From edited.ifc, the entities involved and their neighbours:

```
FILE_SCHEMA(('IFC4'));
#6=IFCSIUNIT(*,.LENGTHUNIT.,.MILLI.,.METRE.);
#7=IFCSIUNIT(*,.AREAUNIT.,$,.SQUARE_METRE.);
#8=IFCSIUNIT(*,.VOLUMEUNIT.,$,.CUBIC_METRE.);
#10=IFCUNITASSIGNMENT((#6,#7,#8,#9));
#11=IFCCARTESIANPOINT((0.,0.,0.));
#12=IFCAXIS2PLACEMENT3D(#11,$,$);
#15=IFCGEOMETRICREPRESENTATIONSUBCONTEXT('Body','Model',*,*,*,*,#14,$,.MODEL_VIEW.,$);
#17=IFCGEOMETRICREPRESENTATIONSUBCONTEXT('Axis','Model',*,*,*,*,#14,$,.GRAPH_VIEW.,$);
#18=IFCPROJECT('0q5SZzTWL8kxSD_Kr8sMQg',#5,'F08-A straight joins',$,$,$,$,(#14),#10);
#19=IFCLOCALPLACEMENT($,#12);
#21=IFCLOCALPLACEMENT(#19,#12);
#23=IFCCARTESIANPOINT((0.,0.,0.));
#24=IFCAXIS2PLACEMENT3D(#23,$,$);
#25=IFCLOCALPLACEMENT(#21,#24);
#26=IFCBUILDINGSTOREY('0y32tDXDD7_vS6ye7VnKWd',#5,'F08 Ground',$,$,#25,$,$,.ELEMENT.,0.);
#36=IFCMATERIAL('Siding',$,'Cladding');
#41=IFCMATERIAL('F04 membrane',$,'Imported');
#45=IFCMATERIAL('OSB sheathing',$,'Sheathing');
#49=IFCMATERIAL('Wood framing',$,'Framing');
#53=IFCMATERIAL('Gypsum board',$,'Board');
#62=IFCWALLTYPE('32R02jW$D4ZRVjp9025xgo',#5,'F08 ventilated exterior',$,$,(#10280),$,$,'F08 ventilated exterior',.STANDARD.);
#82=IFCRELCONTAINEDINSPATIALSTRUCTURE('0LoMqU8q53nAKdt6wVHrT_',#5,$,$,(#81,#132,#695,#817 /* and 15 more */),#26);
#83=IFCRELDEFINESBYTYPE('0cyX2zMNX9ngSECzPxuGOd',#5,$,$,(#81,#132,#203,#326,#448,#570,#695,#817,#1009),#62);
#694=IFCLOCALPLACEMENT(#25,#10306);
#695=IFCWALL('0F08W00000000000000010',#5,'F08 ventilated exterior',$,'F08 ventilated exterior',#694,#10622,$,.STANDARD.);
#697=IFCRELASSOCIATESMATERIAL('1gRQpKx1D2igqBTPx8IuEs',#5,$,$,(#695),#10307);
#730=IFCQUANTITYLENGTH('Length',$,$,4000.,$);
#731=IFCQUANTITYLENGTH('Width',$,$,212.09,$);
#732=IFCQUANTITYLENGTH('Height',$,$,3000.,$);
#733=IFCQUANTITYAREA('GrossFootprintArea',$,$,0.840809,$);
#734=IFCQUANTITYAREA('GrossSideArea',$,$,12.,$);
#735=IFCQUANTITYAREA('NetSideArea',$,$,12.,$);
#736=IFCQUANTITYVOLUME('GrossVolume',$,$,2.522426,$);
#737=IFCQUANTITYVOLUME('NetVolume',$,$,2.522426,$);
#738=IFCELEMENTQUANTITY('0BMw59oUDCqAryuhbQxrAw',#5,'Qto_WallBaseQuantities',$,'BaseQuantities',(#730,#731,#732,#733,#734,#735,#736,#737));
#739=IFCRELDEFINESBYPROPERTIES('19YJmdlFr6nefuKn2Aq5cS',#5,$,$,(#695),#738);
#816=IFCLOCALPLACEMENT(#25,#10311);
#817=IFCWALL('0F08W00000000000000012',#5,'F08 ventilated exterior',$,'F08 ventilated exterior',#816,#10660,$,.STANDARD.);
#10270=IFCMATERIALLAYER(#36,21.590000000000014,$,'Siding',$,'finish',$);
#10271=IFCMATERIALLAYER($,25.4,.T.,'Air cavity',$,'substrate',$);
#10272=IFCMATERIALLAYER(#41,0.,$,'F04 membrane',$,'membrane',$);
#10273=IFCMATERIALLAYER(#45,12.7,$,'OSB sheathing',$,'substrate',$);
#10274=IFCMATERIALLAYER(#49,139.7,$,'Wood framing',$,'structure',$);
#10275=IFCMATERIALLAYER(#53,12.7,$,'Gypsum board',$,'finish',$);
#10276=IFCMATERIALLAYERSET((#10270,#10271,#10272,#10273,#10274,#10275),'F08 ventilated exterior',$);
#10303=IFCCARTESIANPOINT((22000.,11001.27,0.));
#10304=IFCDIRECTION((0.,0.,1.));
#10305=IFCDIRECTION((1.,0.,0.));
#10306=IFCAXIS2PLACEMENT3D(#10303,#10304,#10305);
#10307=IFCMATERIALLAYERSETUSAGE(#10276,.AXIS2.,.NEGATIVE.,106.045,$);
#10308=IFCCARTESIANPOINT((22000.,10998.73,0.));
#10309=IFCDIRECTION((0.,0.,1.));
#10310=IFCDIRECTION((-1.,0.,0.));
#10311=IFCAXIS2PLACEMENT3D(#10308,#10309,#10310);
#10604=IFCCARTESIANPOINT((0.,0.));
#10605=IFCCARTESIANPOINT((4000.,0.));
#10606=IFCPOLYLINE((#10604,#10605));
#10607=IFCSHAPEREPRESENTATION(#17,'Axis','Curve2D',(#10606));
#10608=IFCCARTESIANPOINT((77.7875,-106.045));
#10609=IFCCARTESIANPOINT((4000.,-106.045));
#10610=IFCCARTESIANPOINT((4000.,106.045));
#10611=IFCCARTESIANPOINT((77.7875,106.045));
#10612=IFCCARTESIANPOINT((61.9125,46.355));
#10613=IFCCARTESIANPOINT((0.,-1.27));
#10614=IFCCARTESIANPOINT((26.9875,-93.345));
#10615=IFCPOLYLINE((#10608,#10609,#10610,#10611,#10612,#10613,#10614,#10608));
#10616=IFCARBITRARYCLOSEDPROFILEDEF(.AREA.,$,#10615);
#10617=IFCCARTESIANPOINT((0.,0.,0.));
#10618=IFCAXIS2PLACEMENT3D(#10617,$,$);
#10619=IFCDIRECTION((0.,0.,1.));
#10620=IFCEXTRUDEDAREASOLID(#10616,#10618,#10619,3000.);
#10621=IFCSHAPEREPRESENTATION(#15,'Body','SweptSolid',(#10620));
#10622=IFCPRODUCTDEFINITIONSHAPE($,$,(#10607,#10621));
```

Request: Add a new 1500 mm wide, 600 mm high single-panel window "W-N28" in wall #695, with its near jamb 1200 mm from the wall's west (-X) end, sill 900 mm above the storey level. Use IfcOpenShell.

```python
import numpy as np
import ifcopenshell
import ifcopenshell.api.feature
import ifcopenshell.api.geometry
import ifcopenshell.api.pset
import ifcopenshell.api.root
import ifcopenshell.api.spatial
import ifcopenshell.geom
import ifcopenshell.util.element
import ifcopenshell.util.placement
import ifcopenshell.util.representation
import ifcopenshell.util.shape
import ifcopenshell.util.unit

model = ifcopenshell.open("edited.ifc")
unit_scale = ifcopenshell.util.unit.calculate_unit_scale(model)
area_scale = ifcopenshell.util.unit.calculate_unit_scale(model, "AREAUNIT")
volume_scale = ifcopenshell.util.unit.calculate_unit_scale(model, "VOLUMEUNIT")
settings = ifcopenshell.geom.settings()


def volume(element):
    """Net volume in cubic metres, openings subtracted."""
    shape = ifcopenshell.geom.create_shape(settings, element)
    return ifcopenshell.util.shape.get_volume(shape.geometry)


wall = model.by_guid("0F08W00000000000000010")
storey = ifcopenshell.util.element.get_container(wall, ifc_class="IfcBuildingStorey")
context = ifcopenshell.util.representation.get_context(model, "Model", "Body", "MODEL_VIEW")
before = volume(wall)

width, height, from_end, sill = 1.5, 0.6, 1.2, 0.9  # metres

# The wall runs along its own X axis, and the end named is its -X end.
wall_shape = ifcopenshell.geom.create_shape(settings, wall)
x, y, z = ifcopenshell.util.shape.get_vertices(wall_shape.geometry).T
start = x.min() + from_end
face, thickness = float(y.min()), float(y.max() - y.min())
wall_matrix = ifcopenshell.util.placement.get_local_placement(wall.ObjectPlacement)
level = ifcopenshell.util.placement.get_local_placement(storey.ObjectPlacement)[2, 3]


def in_wall(x, y):
    """Placement at x, y metres in the wall's axes, at sill height."""
    matrix = wall_matrix.copy()
    matrix[:, 3] = wall_matrix @ np.array([x / unit_scale, y / unit_scale, 0.0, 1.0])
    matrix[2, 3] = level + sill / unit_scale
    return matrix


# Opening: a box that overshoots both wall faces by 50 mm.
opening = ifcopenshell.api.root.create_entity(model, ifc_class="IfcOpeningElement", predefined_type="OPENING")
box = ifcopenshell.api.geometry.add_wall_representation(
    model, context=context, length=width, height=height, thickness=thickness + 0.1
)
ifcopenshell.api.geometry.assign_representation(model, product=opening, representation=box)
ifcopenshell.api.geometry.edit_object_placement(model, product=opening, matrix=in_wall(start, face - 0.05), is_si=False)
ifcopenshell.api.feature.add_feature(model, feature=opening, element=wall)

window = ifcopenshell.api.root.create_entity(model, ifc_class="IfcWindow", name="W-N28", predefined_type="WINDOW")
window.OverallWidth, window.OverallHeight = width / unit_scale, height / unit_scale
window.PartitioningType = "SINGLE_PANEL"
body = ifcopenshell.api.geometry.add_window_representation(
    model,
    context=context,
    overall_width=window.OverallWidth,
    overall_height=window.OverallHeight,
    partition_type="SINGLE_PANEL",
)
ifcopenshell.api.geometry.assign_representation(model, product=window, representation=body)
ifcopenshell.api.spatial.assign_container(model, products=[window], relating_structure=storey)
ifcopenshell.api.feature.add_filling(model, opening=opening, element=window)

# Centre the window in the wall's thickness.
ifcopenshell.api.geometry.edit_object_placement(model, product=window, matrix=in_wall(start, face), is_si=False)
window_shape = ifcopenshell.geom.create_shape(settings, window)
depth = ifcopenshell.util.shape.get_vertices(window_shape.geometry)[:, 1]
offset = face + thickness / 2 - (depth.min() + depth.max()) / 2
ifcopenshell.api.geometry.edit_object_placement(model, product=window, matrix=in_wall(start, offset), is_si=False)

after = volume(wall)

# Update the wall's stored quantities.
qto = model.by_id(ifcopenshell.util.element.get_pset(wall, "Qto_WallBaseQuantities", should_inherit=False)["id"])
ifcopenshell.api.pset.edit_qto(model, qto=qto, properties={
    "NetSideArea": after / thickness / area_scale,
    "NetVolume": after / volume_scale,
})

print(f"wall volume {before:.3f} -> {after:.3f} m3")

model.write("edited_v2.ifc")
```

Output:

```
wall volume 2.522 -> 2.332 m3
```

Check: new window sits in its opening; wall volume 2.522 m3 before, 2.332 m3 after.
